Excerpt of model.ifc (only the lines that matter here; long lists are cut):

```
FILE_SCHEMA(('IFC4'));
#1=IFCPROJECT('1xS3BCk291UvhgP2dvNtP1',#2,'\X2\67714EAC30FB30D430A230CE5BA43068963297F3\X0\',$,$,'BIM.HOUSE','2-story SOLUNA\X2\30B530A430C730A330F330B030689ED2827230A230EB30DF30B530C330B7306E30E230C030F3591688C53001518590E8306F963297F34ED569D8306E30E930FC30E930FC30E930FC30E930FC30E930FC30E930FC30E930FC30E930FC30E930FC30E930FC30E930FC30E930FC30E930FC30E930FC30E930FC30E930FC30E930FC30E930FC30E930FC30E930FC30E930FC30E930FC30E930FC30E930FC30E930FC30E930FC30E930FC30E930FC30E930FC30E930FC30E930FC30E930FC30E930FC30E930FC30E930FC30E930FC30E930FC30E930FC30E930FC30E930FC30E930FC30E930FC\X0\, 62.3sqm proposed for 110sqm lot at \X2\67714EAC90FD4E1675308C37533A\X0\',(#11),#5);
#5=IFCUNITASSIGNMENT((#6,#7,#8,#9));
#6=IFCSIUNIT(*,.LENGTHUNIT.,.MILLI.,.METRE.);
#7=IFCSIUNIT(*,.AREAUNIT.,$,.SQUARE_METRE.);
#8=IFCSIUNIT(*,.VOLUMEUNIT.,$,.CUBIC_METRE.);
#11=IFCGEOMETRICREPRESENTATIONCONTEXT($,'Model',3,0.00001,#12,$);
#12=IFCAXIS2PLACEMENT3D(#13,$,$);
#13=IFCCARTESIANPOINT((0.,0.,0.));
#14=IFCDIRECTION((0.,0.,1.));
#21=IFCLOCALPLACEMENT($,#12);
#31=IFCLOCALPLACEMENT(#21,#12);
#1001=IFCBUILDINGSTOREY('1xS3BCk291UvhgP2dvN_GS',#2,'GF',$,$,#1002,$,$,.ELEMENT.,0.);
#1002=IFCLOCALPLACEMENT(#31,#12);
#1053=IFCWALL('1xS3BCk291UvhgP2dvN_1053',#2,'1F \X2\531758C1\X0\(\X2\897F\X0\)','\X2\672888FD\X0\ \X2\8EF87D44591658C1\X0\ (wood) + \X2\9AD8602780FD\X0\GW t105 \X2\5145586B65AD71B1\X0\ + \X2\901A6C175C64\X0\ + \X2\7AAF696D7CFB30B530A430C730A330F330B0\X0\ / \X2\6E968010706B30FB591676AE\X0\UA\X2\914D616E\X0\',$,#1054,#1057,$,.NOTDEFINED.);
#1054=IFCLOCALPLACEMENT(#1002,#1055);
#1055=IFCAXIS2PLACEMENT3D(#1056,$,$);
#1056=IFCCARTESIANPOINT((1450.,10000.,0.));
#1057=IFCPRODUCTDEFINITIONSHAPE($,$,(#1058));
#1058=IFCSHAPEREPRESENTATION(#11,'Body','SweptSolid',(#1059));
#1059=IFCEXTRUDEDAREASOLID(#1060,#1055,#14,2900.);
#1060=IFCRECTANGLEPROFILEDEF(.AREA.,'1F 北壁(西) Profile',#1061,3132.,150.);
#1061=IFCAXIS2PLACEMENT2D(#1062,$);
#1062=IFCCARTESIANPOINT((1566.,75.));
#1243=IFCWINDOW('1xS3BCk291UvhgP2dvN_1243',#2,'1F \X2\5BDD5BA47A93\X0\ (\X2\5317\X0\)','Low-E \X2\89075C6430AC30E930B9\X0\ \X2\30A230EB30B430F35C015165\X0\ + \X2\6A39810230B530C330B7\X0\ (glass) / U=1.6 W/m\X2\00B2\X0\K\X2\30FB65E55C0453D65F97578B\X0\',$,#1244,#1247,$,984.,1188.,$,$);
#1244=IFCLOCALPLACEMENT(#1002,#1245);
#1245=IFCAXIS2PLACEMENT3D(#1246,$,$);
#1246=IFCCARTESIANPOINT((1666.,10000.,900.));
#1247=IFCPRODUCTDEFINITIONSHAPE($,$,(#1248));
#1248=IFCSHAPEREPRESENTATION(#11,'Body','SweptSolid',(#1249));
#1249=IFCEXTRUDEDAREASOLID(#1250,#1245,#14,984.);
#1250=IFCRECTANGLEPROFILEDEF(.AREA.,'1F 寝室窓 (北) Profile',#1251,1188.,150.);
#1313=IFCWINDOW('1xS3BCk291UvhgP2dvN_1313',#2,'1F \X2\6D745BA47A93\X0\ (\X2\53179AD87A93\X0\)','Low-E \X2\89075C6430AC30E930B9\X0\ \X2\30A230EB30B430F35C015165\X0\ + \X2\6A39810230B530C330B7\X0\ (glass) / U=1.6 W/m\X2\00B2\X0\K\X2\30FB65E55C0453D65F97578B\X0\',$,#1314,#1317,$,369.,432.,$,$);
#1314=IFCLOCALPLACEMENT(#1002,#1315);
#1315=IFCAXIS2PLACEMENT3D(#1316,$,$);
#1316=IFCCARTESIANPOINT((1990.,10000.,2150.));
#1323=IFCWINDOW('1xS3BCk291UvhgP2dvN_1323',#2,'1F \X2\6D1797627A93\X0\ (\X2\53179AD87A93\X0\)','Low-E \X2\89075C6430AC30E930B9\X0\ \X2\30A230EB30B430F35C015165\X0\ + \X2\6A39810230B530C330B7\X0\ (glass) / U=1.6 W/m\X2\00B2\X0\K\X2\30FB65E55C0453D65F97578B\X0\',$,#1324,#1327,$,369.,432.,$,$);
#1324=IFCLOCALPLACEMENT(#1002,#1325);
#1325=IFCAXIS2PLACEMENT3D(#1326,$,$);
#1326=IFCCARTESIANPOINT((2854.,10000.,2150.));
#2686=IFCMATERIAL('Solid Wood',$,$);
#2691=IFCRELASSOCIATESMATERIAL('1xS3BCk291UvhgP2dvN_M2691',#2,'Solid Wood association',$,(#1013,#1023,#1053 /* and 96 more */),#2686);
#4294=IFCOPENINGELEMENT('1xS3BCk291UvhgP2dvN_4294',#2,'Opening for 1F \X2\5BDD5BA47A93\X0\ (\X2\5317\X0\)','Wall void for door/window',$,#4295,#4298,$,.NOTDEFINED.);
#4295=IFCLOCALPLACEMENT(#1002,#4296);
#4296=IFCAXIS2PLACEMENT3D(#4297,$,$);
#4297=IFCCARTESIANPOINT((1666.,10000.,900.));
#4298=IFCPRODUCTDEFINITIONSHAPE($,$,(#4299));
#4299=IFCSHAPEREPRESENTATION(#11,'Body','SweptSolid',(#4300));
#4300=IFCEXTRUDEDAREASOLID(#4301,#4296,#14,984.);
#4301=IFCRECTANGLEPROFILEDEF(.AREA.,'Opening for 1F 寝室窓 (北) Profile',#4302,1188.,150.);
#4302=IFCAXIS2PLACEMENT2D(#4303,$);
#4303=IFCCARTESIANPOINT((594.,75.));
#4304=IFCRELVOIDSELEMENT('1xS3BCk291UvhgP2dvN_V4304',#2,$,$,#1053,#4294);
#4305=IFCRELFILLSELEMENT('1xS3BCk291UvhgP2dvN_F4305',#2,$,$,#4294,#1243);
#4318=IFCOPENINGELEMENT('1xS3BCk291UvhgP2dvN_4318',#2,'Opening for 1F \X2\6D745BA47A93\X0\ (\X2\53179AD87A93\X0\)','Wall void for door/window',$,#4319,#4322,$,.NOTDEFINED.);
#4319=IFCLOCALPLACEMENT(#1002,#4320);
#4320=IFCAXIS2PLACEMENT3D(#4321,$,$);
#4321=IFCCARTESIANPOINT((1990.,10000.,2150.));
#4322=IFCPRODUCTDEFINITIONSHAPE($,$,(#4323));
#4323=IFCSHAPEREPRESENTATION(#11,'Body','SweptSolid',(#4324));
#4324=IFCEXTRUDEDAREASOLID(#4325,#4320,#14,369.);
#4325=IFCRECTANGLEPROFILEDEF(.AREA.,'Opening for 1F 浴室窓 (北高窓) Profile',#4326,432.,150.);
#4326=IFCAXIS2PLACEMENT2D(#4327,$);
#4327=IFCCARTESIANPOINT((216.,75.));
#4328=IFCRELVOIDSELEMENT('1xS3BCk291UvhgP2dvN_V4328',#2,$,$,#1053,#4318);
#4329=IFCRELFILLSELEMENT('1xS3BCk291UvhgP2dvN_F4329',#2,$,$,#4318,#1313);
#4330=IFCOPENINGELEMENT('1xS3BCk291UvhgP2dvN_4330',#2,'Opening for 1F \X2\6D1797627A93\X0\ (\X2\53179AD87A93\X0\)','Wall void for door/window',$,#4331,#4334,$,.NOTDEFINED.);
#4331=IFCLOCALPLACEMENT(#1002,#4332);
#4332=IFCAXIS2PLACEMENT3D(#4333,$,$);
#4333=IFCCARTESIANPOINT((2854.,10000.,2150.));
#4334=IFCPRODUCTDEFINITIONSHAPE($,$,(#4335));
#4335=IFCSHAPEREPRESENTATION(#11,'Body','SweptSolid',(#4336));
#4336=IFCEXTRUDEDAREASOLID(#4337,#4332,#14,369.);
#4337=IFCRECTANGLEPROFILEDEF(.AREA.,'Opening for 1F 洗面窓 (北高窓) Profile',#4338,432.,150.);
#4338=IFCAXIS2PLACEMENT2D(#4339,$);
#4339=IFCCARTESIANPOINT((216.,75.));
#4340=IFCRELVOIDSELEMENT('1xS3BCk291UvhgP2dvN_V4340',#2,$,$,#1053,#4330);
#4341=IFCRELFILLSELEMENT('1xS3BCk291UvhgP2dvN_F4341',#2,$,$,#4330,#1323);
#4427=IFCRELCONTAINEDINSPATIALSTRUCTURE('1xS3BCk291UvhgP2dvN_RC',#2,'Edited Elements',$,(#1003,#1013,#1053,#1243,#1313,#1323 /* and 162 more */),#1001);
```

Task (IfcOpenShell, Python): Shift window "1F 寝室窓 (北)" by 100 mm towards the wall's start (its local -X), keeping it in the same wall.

```python
import ifcopenshell
import ifcopenshell.api.geometry
import ifcopenshell.util.placement
import ifcopenshell.util.unit

model = ifcopenshell.open("model.ifc")
unit_scale = ifcopenshell.util.unit.calculate_unit_scale(model)

window = model.by_guid("1xS3BCk291UvhgP2dvN_1243")
opening = window.FillsVoids[0].RelatingOpeningElement
wall = opening.VoidsElements[0].RelatingBuildingElement

wall_matrix = ifcopenshell.util.placement.get_local_placement(wall.ObjectPlacement)
shift = wall_matrix[:3, 0] * -0.1 / unit_scale
before = ifcopenshell.util.placement.get_local_placement(window.ObjectPlacement)[:3, 3].copy()

# The window is not placed relative to its opening, so move both.
for product in (opening, window):
    matrix = ifcopenshell.util.placement.get_local_placement(product.ObjectPlacement)
    matrix[:3, 3] += shift
    ifcopenshell.api.geometry.edit_object_placement(model, product=product, matrix=matrix, is_si=False)

after = ifcopenshell.util.placement.get_local_placement(window.ObjectPlacement)[:3, 3]
print("window moved by", (after - before).round(3) + 0.0)

model.write("model-out.ifc")
```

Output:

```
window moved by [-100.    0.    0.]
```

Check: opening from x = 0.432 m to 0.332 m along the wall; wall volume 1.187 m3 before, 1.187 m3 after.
